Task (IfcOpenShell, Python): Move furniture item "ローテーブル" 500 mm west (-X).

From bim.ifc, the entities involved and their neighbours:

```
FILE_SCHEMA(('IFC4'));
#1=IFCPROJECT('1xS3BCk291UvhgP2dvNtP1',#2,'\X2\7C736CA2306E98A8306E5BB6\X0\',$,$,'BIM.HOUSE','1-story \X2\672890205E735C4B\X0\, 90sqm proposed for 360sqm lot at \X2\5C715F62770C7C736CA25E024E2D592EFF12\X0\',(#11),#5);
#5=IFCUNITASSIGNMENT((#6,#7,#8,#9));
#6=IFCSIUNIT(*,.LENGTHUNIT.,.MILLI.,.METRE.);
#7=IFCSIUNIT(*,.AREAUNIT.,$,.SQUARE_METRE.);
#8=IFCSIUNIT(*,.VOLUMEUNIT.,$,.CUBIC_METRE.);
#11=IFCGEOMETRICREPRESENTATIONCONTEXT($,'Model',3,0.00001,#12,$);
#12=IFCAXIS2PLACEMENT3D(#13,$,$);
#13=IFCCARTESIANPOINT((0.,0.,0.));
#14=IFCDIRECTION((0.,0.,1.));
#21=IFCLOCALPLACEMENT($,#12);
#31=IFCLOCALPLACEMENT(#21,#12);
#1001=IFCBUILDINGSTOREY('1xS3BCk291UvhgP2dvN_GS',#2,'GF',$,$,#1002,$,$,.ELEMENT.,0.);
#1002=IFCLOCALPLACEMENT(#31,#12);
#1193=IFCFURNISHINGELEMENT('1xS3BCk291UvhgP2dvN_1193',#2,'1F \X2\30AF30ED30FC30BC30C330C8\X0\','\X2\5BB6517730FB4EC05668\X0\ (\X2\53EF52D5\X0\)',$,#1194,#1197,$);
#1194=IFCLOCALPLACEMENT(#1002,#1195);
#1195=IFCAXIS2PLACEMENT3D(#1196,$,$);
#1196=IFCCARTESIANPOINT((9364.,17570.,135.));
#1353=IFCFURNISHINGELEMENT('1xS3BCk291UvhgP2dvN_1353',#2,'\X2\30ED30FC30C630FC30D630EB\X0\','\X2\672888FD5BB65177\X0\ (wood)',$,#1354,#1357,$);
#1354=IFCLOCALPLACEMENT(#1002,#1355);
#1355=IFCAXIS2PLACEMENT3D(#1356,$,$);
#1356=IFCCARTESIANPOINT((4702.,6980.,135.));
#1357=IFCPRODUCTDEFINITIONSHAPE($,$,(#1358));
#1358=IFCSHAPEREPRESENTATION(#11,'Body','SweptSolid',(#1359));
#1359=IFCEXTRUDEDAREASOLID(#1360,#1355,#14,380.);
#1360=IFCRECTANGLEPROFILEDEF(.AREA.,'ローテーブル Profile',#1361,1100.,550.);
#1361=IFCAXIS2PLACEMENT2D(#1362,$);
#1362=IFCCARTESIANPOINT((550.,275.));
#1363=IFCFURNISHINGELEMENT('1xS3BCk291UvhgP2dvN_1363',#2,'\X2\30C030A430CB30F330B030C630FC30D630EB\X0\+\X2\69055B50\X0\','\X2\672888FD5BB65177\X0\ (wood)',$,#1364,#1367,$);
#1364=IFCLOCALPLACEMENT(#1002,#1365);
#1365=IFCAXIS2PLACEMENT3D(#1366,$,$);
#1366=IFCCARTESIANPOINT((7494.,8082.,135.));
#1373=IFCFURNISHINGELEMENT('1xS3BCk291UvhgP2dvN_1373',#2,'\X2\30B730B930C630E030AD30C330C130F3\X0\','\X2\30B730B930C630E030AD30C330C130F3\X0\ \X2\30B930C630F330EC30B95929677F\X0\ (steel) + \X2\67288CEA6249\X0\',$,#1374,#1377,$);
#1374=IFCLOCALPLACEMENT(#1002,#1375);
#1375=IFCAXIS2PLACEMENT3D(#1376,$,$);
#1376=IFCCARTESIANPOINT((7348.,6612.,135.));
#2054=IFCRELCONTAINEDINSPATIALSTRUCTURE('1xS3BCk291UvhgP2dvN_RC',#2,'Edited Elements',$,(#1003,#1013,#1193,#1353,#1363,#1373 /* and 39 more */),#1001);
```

```python
import ifcopenshell
import ifcopenshell.api.geometry
import ifcopenshell.util.placement

model = ifcopenshell.open("bim.ifc")

item = model.by_guid("1xS3BCk291UvhgP2dvN_1353")
matrix = ifcopenshell.util.placement.get_local_placement(item.ObjectPlacement)
matrix[0, 3] -= 500.0
ifcopenshell.api.geometry.edit_object_placement(model, product=item, matrix=matrix, is_si=False)

print(ifcopenshell.util.placement.get_local_placement(item.ObjectPlacement).round(3) + 0.0)

model.write("bim_v2.ifc")
```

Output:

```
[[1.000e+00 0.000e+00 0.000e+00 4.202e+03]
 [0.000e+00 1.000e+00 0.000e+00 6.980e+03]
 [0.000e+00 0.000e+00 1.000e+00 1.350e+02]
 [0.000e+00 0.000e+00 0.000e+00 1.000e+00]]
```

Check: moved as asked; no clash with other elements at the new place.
